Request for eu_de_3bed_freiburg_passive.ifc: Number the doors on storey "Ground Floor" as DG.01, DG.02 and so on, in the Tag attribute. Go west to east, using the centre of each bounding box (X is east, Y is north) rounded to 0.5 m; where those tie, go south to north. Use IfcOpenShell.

First a look at what the model holds.

```python
import ifcopenshell
import ifcopenshell.util.element
import ifcopenshell.util.placement

model = ifcopenshell.open("eu_de_3bed_freiburg_passive.ifc")
print(model.schema)
storey = next(s for s in model.by_type("IfcBuildingStorey") if s.Name == "Ground Floor")
doors = [e for e in ifcopenshell.util.element.get_decomposition(storey) if e.is_a("IfcDoor")]
for e in sorted(doors, key=lambda e: e.id()):
    origin = ifcopenshell.util.placement.get_local_placement(e.ObjectPlacement)[:3, 3]
    print(e.id(), e.Tag, e.Name, origin.round(2) + 0.0, sep=" | ")
```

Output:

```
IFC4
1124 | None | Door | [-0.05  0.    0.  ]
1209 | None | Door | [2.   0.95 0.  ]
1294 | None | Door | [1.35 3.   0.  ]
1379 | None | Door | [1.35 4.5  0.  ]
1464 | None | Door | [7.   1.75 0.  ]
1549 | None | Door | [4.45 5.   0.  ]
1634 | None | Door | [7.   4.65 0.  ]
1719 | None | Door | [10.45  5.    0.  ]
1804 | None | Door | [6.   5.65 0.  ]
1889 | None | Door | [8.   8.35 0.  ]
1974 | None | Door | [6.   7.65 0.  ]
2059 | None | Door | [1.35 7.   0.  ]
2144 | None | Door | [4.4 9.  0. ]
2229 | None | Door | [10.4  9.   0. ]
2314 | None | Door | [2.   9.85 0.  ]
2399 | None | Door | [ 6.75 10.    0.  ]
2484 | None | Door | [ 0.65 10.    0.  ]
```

```python
import ifcopenshell
import ifcopenshell.geom
import ifcopenshell.util.element
import ifcopenshell.util.shape

model = ifcopenshell.open("eu_de_3bed_freiburg_passive.ifc")
settings = ifcopenshell.geom.settings()
settings.set("use-world-coords", True)


def centre(element):
    shape = ifcopenshell.geom.create_shape(settings, element)
    return ifcopenshell.util.shape.get_bbox_centroid(shape.geometry)


storey = next(s for s in model.by_type("IfcBuildingStorey") if s.Name == "Ground Floor")
doors = [e for e in ifcopenshell.util.element.get_decomposition(storey) if e.is_a("IfcDoor")]

# Insertion points can sit at a corner or the storey origin, so sort by the geometry (in metres).
centres = {e: centre(e) for e in doors}
doors.sort(key=lambda e: (round(centres[e][0] / 0.5), centres[e][1]))

for i, e in enumerate(doors, start=1):
    number = f"DG.{i:02d}"
    e.Tag = number
    print(e.id(), number)

model.write("eu_de_3bed_freiburg_passive_v2.ifc")
```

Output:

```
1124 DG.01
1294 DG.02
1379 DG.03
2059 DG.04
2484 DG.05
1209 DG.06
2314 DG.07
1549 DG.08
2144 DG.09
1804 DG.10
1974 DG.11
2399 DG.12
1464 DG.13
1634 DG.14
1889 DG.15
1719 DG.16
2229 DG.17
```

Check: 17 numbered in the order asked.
